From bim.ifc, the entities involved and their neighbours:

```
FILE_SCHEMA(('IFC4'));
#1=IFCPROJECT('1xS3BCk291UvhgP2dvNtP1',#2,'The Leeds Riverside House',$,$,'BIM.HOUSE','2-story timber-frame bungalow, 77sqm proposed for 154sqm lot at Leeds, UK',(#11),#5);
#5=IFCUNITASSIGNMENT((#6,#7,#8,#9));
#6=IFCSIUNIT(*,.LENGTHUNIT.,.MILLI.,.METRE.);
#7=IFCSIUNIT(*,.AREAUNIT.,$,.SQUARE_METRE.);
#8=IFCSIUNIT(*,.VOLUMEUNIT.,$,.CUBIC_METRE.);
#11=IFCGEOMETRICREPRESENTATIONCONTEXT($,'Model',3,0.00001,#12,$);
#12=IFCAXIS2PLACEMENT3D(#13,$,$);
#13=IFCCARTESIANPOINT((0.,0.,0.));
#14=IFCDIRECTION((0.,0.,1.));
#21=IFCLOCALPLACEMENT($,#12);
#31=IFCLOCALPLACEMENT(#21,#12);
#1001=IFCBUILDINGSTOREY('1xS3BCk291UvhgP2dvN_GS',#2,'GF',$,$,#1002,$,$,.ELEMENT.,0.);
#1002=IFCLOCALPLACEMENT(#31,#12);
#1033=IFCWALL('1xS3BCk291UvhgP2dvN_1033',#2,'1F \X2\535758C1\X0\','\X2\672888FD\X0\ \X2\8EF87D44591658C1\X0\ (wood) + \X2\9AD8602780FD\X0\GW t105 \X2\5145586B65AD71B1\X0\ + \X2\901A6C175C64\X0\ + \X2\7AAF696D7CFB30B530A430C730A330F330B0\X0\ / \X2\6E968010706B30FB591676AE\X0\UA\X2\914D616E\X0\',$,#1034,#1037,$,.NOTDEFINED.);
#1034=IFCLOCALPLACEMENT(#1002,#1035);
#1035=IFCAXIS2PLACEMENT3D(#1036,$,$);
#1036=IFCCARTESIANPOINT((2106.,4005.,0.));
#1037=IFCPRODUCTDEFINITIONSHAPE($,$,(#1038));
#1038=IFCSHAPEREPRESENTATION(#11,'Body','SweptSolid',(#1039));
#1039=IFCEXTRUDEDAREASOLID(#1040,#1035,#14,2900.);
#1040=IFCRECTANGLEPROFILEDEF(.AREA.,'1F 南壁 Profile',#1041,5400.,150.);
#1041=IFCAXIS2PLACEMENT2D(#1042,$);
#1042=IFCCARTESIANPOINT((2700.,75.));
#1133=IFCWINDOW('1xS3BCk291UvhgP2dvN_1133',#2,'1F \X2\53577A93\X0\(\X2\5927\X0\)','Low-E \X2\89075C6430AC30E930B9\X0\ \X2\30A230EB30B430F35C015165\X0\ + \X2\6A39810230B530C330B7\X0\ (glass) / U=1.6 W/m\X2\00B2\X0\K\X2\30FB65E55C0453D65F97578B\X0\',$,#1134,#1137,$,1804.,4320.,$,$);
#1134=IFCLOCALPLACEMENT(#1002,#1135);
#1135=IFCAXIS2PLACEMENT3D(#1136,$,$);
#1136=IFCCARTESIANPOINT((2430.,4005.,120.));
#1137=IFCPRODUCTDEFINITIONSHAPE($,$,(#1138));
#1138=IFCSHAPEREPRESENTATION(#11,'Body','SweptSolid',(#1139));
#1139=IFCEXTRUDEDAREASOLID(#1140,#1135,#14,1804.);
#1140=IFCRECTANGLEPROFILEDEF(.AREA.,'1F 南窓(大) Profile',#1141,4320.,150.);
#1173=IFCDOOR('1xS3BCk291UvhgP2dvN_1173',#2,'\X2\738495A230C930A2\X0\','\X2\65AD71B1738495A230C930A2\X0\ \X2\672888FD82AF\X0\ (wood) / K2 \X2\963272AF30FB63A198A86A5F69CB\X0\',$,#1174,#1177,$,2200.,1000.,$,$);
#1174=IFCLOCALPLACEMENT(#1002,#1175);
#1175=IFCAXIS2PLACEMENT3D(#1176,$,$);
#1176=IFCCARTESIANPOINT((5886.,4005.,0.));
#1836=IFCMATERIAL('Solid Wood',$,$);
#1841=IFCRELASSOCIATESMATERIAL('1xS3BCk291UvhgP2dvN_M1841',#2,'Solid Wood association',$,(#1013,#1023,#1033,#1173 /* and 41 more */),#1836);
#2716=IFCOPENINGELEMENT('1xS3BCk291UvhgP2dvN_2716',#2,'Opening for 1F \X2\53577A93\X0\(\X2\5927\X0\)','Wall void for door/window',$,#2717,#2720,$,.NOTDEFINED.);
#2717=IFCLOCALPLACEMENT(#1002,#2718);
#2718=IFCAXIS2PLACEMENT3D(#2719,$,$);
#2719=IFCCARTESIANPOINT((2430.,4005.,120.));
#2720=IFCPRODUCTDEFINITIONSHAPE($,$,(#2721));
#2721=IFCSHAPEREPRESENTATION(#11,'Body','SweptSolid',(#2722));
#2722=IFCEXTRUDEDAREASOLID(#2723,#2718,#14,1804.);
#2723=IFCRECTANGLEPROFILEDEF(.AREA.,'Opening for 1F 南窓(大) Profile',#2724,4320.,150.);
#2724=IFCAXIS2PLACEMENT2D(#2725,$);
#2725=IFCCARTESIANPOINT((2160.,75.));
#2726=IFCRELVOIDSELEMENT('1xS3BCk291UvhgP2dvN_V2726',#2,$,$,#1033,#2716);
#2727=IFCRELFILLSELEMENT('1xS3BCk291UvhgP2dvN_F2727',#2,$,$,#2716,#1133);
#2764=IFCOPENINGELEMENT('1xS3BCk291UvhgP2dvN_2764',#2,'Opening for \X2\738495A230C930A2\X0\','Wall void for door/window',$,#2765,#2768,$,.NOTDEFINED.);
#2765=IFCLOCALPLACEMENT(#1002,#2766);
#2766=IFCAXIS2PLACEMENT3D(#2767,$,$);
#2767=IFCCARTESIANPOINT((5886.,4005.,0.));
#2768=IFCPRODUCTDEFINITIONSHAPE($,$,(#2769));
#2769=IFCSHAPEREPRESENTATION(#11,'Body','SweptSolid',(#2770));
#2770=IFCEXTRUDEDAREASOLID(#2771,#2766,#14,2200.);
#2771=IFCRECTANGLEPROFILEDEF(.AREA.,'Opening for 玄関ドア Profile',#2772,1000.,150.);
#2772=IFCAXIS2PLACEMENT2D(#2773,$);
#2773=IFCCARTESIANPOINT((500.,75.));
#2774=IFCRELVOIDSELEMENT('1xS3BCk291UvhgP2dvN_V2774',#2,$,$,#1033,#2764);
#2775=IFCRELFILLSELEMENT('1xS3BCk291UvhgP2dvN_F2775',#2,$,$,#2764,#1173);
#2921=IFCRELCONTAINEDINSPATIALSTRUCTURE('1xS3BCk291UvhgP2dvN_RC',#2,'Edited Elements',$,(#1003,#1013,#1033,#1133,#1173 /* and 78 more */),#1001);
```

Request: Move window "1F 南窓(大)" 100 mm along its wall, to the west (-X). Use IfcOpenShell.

```python
import ifcopenshell
import ifcopenshell.api.geometry
import ifcopenshell.util.placement
import ifcopenshell.util.unit

model = ifcopenshell.open("bim.ifc")
unit_scale = ifcopenshell.util.unit.calculate_unit_scale(model)

window = model.by_guid("1xS3BCk291UvhgP2dvN_1133")
opening = window.FillsVoids[0].RelatingOpeningElement
wall = opening.VoidsElements[0].RelatingBuildingElement

wall_matrix = ifcopenshell.util.placement.get_local_placement(wall.ObjectPlacement)
shift = wall_matrix[:3, 0] * -0.1 / unit_scale
before = ifcopenshell.util.placement.get_local_placement(window.ObjectPlacement)[:3, 3].copy()

# The window is not placed relative to its opening, so move both.
for product in (opening, window):
    matrix = ifcopenshell.util.placement.get_local_placement(product.ObjectPlacement)
    matrix[:3, 3] += shift
    ifcopenshell.api.geometry.edit_object_placement(model, product=product, matrix=matrix, is_si=False)

after = ifcopenshell.util.placement.get_local_placement(window.ObjectPlacement)[:3, 3]
print("window moved by", (after - before).round(3) + 0.0)

model.write("bim_edited.ifc")
```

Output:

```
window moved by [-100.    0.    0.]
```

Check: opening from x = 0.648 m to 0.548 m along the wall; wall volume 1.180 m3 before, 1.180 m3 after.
